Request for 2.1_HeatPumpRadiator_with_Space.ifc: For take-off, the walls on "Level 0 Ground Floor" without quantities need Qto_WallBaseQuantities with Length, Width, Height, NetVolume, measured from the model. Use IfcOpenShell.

First a look at what the model holds.

```python
import ifcopenshell
import ifcopenshell.util.element
import ifcopenshell.util.unit

model = ifcopenshell.open("2.1_HeatPumpRadiator_with_Space.ifc")
print(model.schema)
for unit_type in ("LENGTHUNIT", "AREAUNIT", "VOLUMEUNIT"):
    print(unit_type, ifcopenshell.util.unit.calculate_unit_scale(model, unit_type))
storey = next(s for s in model.by_type("IfcBuildingStorey") if s.Name == "Level 0 Ground Floor")
walls = [e for e in ifcopenshell.util.element.get_decomposition(storey) if e.is_a("IfcWall")]
for e in sorted(walls, key=lambda e: e.id()):
    print(e.id(), e.is_a(), e.Name, list(ifcopenshell.util.element.get_psets(e, qtos_only=True)), sep=" | ")
```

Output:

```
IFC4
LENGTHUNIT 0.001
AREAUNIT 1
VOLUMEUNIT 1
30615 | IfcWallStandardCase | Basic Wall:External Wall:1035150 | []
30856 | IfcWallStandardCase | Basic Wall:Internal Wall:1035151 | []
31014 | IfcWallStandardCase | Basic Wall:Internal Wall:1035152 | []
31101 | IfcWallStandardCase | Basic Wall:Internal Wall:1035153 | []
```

```python
import ifcopenshell
import ifcopenshell.api.pset
import ifcopenshell.geom
import ifcopenshell.util.element
import ifcopenshell.util.shape
import ifcopenshell.util.unit

model = ifcopenshell.open("2.1_HeatPumpRadiator_with_Space.ifc")
unit_scale = ifcopenshell.util.unit.calculate_unit_scale(model)
volume_scale = ifcopenshell.util.unit.calculate_unit_scale(model, "VOLUMEUNIT")
settings = ifcopenshell.geom.settings()

storey = next(s for s in model.by_type("IfcBuildingStorey") if s.Name == "Level 0 Ground Floor")
walls = [e for e in ifcopenshell.util.element.get_decomposition(storey) if e.is_a("IfcWall")]

for e in sorted(walls, key=lambda e: e.id()):
    if ifcopenshell.util.element.get_psets(e, qtos_only=True, should_inherit=False):
        continue
    # Geometry comes back in metres, in the element's own axes.
    shape = ifcopenshell.geom.create_shape(settings, e)
    values = {
        "Length": ifcopenshell.util.shape.get_x(shape.geometry) / unit_scale,
        "Width": ifcopenshell.util.shape.get_y(shape.geometry) / unit_scale,
        "Height": ifcopenshell.util.shape.get_z(shape.geometry) / unit_scale,
        "NetVolume": ifcopenshell.util.shape.get_volume(shape.geometry) / volume_scale,
    }
    qto = ifcopenshell.api.pset.add_qto(model, product=e, name="Qto_WallBaseQuantities")
    ifcopenshell.api.pset.edit_qto(model, qto=qto, properties=values)
    print(e.id(), {k: round(v, 3) for k, v in values.items()})

model.write("2.1_HeatPumpRadiator_with_Space_edited.ifc")
```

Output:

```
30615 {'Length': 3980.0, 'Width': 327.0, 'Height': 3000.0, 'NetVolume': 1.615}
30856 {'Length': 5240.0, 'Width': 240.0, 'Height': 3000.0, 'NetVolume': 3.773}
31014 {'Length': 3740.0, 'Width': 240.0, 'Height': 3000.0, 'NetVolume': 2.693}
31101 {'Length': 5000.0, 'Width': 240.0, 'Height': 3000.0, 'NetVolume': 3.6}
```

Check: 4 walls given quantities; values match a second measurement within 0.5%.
